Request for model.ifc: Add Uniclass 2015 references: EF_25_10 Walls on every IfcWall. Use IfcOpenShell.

First a look at what the model holds.

```python
import ifcopenshell

model = ifcopenshell.open("model.ifc")
print(model.schema)
print("classifications:", [c.Name for c in model.by_type("IfcClassification")])
for ifc_class in ("IfcDoor", "IfcRoof", "IfcStair", "IfcWall", "IfcWindow"):
    print(ifc_class, len(model.by_type(ifc_class)))
```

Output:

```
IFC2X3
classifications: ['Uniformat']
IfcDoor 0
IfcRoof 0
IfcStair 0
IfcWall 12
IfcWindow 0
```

```python
import ifcopenshell
import ifcopenshell.api.classification

model = ifcopenshell.open("model.ifc")

# IFC2X3 requires Source and Edition and has no link from the project to the system.
system = model.create_entity("IfcClassification", Source="NBS", Edition="2015", Name="Uniclass 2015")

codes = {
    "IfcWall": ("EF_25_10", "Walls"),
}
for ifc_class, (code, name) in codes.items():
    products = model.by_type(ifc_class)
    ifcopenshell.api.classification.add_reference(
        model, products=products, classification=system, identification=code, name=name
    )
    print(code, len(products))

model.write("model_v2.ifc")
```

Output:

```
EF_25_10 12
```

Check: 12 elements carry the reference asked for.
